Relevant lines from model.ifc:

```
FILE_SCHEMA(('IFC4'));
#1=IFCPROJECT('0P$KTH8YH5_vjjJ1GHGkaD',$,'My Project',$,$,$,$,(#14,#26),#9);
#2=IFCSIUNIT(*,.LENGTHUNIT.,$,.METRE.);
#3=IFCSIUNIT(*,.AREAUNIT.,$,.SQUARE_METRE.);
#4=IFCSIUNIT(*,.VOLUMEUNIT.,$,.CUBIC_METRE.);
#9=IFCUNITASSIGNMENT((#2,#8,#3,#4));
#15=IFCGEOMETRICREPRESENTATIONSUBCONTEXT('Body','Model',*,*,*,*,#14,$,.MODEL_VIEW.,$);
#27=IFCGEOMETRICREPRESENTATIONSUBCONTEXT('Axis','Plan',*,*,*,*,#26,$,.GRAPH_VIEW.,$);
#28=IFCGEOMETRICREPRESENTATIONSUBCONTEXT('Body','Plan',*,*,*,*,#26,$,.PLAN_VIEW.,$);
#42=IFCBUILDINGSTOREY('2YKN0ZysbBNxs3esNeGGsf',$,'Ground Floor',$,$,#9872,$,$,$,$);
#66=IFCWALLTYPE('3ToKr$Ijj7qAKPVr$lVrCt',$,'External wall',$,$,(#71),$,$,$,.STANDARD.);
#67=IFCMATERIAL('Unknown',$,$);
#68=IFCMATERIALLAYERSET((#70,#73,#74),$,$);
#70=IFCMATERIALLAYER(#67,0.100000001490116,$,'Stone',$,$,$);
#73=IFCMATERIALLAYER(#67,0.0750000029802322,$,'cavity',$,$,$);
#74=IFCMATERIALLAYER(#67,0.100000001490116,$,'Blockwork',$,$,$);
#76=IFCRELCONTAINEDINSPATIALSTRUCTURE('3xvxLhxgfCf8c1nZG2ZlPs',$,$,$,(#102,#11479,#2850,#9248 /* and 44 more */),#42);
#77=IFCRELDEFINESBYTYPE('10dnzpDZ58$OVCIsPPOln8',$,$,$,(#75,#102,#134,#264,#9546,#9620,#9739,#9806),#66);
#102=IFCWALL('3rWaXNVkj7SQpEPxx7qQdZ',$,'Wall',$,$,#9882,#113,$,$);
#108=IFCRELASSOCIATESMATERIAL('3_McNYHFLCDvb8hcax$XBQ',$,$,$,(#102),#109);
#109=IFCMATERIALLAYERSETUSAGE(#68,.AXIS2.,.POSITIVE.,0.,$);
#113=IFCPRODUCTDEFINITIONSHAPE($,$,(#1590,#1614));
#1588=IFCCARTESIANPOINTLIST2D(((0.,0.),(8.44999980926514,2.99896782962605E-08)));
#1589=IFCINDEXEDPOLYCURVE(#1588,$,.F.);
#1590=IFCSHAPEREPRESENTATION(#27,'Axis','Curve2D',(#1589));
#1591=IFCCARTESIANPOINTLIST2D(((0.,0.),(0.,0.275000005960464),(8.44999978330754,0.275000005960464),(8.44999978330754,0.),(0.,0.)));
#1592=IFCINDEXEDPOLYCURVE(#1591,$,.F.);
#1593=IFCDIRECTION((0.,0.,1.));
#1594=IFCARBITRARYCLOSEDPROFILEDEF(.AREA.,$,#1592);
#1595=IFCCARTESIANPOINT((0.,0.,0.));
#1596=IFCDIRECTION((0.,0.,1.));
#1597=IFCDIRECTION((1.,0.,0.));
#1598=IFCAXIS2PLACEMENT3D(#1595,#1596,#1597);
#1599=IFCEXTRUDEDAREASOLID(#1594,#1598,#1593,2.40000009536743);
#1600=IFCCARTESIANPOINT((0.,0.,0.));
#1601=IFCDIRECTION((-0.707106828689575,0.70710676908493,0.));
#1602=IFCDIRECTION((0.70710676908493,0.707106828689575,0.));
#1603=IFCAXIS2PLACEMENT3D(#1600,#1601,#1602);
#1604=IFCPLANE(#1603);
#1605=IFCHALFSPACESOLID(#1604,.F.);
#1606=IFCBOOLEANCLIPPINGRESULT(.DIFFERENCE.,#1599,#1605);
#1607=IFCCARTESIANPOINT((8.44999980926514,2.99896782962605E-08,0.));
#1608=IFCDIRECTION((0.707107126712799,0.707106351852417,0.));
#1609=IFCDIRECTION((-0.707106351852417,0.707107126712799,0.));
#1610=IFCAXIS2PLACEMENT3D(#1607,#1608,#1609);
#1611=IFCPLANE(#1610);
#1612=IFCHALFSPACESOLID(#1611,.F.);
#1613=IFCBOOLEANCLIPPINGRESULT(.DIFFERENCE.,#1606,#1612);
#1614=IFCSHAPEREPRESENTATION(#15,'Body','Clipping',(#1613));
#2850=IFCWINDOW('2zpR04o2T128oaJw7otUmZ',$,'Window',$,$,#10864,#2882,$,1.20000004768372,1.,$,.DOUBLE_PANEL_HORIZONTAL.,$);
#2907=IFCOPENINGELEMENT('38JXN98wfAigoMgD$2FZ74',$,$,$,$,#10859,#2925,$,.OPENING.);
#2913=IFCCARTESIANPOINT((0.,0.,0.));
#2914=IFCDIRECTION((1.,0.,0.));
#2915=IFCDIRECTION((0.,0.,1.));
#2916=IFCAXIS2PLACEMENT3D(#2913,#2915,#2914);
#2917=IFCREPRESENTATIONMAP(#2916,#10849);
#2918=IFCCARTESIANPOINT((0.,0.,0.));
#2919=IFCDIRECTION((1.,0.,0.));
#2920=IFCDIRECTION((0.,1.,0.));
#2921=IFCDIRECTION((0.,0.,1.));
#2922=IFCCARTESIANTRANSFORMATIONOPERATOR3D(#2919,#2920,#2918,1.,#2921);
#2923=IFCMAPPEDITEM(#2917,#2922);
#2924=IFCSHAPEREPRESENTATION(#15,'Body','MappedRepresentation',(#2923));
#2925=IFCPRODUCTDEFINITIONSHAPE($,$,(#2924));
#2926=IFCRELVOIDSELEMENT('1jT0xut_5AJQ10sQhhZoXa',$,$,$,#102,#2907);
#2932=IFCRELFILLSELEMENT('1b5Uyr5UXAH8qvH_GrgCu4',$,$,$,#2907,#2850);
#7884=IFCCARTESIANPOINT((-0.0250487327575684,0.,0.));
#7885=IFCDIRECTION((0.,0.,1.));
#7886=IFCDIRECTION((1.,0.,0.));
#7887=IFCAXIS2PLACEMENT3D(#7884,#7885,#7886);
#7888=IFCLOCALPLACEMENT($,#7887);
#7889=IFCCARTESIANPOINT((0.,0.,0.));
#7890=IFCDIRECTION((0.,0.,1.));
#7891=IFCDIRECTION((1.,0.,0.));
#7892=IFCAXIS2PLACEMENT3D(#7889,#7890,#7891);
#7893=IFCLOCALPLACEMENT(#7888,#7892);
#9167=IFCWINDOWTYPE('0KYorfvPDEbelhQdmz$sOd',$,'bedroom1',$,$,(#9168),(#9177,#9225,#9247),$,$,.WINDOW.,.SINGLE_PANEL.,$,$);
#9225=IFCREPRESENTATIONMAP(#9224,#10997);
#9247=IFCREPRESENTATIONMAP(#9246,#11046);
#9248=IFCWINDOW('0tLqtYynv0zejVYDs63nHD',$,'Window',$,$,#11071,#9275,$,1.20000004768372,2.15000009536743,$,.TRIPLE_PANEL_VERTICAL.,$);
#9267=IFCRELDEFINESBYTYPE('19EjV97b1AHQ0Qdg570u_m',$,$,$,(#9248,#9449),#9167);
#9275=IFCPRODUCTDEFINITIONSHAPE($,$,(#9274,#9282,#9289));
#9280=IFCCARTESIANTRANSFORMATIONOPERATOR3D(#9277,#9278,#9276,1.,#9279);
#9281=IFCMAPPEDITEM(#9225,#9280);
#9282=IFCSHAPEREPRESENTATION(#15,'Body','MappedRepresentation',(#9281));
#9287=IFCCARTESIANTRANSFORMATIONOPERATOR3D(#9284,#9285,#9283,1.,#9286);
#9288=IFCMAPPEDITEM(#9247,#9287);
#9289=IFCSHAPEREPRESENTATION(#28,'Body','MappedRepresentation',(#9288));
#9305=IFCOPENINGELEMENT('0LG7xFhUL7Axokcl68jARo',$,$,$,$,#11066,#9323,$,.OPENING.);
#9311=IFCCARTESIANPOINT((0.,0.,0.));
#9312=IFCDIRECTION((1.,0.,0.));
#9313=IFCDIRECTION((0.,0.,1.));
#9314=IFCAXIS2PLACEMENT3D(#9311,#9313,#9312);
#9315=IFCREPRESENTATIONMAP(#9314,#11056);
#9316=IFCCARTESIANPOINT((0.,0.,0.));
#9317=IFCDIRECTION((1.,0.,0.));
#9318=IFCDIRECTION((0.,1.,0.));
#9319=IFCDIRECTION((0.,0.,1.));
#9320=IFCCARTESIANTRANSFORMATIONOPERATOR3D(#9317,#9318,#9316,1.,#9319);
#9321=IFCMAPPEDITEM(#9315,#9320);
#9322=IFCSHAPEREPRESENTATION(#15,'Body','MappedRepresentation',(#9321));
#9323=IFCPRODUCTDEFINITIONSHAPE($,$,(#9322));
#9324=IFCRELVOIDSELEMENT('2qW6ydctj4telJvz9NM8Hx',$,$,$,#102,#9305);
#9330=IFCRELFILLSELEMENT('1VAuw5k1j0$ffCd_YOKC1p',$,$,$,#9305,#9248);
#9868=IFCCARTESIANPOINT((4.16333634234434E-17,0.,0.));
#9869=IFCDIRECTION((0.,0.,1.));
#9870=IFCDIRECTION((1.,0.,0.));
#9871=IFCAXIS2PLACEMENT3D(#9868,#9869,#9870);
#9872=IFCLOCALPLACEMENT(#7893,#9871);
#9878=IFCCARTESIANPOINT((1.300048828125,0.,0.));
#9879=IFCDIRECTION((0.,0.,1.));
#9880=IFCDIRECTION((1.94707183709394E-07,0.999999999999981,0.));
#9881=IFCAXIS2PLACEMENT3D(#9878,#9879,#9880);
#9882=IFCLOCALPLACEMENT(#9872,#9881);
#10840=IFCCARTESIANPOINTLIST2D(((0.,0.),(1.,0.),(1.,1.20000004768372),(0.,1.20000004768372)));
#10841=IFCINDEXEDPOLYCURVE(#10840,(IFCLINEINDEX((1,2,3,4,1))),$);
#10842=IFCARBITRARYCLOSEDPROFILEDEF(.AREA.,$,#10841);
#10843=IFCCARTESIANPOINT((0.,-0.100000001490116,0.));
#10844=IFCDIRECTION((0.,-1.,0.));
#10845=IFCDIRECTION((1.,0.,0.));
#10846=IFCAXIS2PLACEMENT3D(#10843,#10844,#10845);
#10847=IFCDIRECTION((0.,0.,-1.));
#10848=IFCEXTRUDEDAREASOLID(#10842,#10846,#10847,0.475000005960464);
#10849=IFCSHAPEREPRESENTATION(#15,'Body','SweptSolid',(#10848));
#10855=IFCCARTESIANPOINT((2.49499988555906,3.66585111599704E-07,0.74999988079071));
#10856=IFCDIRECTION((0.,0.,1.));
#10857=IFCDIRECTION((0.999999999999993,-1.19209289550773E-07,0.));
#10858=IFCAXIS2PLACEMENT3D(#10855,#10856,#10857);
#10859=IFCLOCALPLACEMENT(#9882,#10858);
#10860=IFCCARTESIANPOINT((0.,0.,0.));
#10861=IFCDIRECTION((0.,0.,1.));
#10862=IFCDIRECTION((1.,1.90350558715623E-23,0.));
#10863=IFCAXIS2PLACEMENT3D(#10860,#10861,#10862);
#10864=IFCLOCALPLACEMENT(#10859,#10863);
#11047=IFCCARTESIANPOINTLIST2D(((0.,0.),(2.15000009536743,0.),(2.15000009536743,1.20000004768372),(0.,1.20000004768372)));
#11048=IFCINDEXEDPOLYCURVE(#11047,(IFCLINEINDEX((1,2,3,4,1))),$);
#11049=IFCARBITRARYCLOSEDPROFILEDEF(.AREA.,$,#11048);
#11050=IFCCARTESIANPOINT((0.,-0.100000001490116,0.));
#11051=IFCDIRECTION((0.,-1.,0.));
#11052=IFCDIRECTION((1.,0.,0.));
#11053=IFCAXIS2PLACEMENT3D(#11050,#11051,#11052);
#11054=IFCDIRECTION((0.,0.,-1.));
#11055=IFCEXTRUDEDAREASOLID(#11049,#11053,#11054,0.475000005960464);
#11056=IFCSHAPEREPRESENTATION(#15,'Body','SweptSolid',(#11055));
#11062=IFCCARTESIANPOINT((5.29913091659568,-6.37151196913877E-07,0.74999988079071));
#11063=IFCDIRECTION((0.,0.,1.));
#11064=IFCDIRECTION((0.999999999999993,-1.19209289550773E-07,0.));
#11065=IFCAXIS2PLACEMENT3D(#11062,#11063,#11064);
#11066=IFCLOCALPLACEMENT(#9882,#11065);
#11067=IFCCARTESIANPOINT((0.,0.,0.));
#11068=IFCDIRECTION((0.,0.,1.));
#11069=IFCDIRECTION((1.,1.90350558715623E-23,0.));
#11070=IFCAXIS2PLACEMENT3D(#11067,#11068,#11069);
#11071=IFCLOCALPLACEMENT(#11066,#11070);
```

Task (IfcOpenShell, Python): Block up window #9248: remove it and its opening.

```python
import ifcopenshell
import ifcopenshell.api.feature
import ifcopenshell.api.root
import ifcopenshell.geom
import ifcopenshell.util.shape

model = ifcopenshell.open("model.ifc")
settings = ifcopenshell.geom.settings()


def volume(element):
    """Net volume in cubic metres, openings subtracted."""
    shape = ifcopenshell.geom.create_shape(settings, element)
    return ifcopenshell.util.shape.get_volume(shape.geometry)


window = model.by_id(9248)
opening = window.FillsVoids[0].RelatingOpeningElement
wall = opening.VoidsElements[0].RelatingBuildingElement
before = volume(wall)

ifcopenshell.api.root.remove_product(model, product=window)
ifcopenshell.api.feature.remove_feature(model, feature=opening)

after = volume(wall)

print(f"wall volume {before:.3f} -> {after:.3f} m3")

model.write("model-out.ifc")
```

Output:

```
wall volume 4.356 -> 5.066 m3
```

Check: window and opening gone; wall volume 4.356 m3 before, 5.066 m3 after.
